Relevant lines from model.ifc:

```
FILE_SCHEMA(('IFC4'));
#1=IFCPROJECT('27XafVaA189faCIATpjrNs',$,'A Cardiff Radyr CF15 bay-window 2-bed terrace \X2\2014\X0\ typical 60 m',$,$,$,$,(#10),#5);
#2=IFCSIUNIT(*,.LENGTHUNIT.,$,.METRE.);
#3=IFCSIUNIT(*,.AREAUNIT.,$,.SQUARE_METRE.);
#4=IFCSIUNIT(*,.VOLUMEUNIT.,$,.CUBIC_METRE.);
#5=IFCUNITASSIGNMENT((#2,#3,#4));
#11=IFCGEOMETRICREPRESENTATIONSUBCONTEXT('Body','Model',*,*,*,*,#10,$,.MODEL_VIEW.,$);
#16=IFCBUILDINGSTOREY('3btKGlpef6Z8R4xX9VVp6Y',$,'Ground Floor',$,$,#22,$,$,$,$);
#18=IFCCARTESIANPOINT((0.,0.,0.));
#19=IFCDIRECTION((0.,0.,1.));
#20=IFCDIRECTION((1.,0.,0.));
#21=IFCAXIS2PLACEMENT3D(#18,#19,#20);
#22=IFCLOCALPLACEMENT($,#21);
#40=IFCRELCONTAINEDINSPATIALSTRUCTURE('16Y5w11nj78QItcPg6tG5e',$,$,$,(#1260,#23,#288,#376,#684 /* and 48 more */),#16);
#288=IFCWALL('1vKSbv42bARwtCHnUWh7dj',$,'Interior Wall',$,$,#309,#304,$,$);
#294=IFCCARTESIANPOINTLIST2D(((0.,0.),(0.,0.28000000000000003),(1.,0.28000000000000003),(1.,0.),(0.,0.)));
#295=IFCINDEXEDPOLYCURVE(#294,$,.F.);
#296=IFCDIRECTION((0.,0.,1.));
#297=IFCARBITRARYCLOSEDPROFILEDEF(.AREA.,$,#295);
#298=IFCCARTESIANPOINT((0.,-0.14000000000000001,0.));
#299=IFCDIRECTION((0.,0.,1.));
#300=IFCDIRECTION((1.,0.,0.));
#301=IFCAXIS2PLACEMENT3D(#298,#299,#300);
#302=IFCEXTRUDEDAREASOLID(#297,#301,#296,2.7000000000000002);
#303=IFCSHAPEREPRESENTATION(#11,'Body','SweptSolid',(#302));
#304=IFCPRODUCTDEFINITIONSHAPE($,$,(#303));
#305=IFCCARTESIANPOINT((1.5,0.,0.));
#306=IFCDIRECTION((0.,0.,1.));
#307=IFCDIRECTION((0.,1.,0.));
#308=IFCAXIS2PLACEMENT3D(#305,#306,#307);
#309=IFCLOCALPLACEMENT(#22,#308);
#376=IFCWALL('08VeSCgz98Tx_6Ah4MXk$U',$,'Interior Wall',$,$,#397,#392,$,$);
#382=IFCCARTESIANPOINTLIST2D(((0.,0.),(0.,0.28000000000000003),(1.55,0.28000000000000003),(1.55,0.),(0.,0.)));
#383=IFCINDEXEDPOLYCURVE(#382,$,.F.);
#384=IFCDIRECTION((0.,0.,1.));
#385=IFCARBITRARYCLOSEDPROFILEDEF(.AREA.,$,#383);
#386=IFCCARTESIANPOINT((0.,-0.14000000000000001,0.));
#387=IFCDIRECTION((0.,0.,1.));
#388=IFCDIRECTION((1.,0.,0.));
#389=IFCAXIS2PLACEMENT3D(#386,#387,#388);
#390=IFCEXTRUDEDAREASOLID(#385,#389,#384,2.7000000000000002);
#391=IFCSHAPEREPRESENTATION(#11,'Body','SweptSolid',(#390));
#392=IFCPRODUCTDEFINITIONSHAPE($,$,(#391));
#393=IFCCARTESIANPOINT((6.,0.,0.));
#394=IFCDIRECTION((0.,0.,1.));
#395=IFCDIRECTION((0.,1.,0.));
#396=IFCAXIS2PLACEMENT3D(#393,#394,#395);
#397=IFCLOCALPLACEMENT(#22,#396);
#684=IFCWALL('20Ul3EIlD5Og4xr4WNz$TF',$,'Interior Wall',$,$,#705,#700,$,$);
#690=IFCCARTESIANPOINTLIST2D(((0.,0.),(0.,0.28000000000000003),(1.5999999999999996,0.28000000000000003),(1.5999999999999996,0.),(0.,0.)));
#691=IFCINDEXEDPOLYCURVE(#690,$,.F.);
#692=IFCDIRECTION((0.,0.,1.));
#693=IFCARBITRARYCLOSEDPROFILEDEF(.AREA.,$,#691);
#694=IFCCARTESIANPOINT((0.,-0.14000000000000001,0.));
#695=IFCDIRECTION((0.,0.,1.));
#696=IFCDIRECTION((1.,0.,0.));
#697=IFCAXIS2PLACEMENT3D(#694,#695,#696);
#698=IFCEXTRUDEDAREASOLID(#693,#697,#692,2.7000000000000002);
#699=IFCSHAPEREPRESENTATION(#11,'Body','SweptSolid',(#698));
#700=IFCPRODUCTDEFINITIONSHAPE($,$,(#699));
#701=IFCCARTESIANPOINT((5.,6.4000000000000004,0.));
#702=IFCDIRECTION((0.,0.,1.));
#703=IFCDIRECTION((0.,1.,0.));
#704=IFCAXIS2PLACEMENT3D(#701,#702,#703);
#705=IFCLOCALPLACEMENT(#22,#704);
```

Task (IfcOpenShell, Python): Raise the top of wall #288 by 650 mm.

```python
import ifcopenshell
import ifcopenshell.geom
import ifcopenshell.util.representation
import ifcopenshell.util.shape
import ifcopenshell.util.unit

model = ifcopenshell.open("model.ifc")
unit_scale = ifcopenshell.util.unit.calculate_unit_scale(model)
settings = ifcopenshell.geom.settings()


def volume(element):
    """Net volume in cubic metres, openings subtracted."""
    shape = ifcopenshell.geom.create_shape(settings, element)
    return ifcopenshell.util.shape.get_volume(shape.geometry)


wall = model.by_guid("1vKSbv42bARwtCHnUWh7dj")
before = volume(wall)

body = ifcopenshell.util.representation.get_representation(wall, "Model", "Body")
solid = body.Items[0]
old_height = solid.Depth
solid.Depth += 0.65 / unit_scale
after = volume(wall)

print(f"height {old_height:g} -> {solid.Depth:g}, volume {before:.3f} -> {after:.3f} m3")

model.write("model_rev.ifc")
```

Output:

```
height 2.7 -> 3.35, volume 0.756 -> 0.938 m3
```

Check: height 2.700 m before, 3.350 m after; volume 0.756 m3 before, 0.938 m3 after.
